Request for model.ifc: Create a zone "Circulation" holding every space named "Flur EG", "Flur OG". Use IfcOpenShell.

First a look at what the model holds.

```python
import ifcopenshell

model = ifcopenshell.open("model.ifc")
print(model.schema)
seen = {}
for space in model.by_type("IfcSpace"):
    seen[space.Name] = seen.get(space.Name, 0) + 1
for name, count in sorted(seen.items(), key=str):
    print(count, "x", name)
print("zones:", [z.Name for z in model.by_type("IfcZone")][:20])
```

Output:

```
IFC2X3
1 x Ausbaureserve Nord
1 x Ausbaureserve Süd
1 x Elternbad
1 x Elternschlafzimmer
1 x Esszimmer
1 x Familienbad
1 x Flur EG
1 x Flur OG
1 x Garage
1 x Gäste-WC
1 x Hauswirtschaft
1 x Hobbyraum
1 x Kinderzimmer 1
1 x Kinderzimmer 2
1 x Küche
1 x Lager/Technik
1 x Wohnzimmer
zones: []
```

```python
import ifcopenshell
import ifcopenshell.api.group
import ifcopenshell.api.root

model = ifcopenshell.open("model.ifc")

names = {"Flur EG", "Flur OG"}
spaces = [s for s in model.by_type("IfcSpace") if s.Name in names]

zone = ifcopenshell.api.root.create_entity(model, ifc_class="IfcZone", name="Circulation")
ifcopenshell.api.group.assign_group(model, products=spaces, group=zone)
print(len(spaces), "spaces in", zone.Name)

model.write("model-out.ifc")
```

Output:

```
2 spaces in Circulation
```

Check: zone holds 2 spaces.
